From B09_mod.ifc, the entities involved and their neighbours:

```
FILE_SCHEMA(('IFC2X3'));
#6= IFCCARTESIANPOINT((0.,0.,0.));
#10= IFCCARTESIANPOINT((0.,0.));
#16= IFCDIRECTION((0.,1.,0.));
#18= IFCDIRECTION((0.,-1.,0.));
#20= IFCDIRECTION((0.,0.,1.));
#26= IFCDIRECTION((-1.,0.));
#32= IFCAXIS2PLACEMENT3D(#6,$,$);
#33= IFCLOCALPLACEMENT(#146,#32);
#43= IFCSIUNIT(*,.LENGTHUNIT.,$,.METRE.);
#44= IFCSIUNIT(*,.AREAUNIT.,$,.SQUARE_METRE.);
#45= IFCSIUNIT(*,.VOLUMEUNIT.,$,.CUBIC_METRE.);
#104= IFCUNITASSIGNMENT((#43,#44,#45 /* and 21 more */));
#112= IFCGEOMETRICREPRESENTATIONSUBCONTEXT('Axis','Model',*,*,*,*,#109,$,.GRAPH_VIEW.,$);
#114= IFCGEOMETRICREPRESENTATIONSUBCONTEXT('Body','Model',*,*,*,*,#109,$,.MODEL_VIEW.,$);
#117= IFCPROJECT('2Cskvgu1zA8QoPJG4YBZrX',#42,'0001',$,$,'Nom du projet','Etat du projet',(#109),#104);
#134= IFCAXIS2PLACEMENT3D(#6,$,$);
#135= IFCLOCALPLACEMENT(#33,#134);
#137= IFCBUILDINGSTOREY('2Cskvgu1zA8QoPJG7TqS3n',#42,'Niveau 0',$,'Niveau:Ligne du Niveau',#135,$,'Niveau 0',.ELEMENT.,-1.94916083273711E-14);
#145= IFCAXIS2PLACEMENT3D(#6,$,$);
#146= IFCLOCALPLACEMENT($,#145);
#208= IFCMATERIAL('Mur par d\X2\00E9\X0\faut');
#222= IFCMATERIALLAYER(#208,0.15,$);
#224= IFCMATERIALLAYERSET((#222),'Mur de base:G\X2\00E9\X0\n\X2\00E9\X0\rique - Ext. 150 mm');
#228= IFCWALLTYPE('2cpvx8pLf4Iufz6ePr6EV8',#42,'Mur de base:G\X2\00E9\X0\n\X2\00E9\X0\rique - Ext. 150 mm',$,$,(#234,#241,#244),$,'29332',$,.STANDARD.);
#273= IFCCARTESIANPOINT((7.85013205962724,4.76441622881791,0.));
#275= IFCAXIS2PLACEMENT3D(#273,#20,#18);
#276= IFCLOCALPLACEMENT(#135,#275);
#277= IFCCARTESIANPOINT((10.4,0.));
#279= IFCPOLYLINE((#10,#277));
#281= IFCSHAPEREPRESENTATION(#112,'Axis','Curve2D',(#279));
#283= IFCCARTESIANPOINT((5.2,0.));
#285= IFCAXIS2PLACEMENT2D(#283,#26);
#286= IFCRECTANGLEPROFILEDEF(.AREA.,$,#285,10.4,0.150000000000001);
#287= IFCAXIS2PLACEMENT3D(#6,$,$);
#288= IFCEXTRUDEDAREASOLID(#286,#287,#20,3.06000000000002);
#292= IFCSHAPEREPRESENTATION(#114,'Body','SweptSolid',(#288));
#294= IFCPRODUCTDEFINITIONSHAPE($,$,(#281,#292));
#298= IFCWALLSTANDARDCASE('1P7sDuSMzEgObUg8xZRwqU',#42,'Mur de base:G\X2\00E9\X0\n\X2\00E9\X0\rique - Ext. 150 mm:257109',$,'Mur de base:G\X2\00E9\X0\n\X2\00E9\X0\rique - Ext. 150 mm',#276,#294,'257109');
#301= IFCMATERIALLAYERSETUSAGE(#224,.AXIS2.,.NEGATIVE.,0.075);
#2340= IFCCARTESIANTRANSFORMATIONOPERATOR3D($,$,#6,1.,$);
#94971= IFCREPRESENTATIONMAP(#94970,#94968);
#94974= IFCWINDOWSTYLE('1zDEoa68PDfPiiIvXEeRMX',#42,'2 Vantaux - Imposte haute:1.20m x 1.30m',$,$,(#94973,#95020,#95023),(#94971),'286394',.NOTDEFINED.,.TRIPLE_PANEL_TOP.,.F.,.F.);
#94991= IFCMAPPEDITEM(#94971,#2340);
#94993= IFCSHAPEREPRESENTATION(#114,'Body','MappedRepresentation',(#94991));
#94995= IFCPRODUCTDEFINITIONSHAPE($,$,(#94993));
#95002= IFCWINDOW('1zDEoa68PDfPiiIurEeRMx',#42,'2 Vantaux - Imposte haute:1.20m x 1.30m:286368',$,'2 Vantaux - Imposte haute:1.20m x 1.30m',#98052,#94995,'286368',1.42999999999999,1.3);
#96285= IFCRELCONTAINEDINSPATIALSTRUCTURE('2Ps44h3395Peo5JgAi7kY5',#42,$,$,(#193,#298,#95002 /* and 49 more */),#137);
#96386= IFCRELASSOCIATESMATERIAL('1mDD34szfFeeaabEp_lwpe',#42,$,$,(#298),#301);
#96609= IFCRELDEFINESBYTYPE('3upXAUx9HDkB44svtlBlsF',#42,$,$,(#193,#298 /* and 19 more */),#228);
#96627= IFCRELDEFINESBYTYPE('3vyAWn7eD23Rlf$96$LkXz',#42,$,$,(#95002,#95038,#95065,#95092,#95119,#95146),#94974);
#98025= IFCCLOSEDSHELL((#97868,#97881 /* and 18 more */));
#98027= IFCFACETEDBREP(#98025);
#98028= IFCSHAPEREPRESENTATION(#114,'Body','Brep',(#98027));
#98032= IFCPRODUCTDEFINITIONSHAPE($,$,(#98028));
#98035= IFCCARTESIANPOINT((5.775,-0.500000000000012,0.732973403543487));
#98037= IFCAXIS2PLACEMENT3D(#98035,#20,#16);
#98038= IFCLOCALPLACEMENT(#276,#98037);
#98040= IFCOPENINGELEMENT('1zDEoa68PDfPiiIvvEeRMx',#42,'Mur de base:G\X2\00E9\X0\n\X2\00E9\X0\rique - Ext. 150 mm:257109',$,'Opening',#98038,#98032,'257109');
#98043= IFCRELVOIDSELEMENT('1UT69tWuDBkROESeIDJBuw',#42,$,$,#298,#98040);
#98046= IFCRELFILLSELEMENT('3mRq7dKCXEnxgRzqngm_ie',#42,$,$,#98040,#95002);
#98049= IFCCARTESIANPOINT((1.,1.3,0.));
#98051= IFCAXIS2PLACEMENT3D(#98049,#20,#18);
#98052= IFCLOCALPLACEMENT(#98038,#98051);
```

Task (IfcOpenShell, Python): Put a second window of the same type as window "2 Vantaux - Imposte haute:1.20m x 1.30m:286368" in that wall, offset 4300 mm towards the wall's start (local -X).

```python
import ifcopenshell
import ifcopenshell.api.feature
import ifcopenshell.api.geometry
import ifcopenshell.api.root
import ifcopenshell.geom
import ifcopenshell.util.element
import ifcopenshell.util.placement
import ifcopenshell.util.shape
import ifcopenshell.util.unit

model = ifcopenshell.open("B09_mod.ifc")
unit_scale = ifcopenshell.util.unit.calculate_unit_scale(model)
settings = ifcopenshell.geom.settings()


def volume(element):
    """Net volume in cubic metres, openings subtracted."""
    shape = ifcopenshell.geom.create_shape(settings, element)
    return ifcopenshell.util.shape.get_volume(shape.geometry)


def reuse_history(source, copy):
    """copy_class also copies each property set's owner history, people and application; keep the originals."""
    for rel in copy.IsDefinedBy:
        if rel.is_a("IfcRelDefinesByProperties") and (history := rel.RelatingPropertyDefinition.OwnerHistory):
            rel.RelatingPropertyDefinition.OwnerHistory = source.OwnerHistory
            ifcopenshell.util.element.remove_deep2(model, history)


window = model.by_guid("1zDEoa68PDfPiiIurEeRMx")
opening = window.FillsVoids[0].RelatingOpeningElement
wall = opening.VoidsElements[0].RelatingBuildingElement
before = volume(wall)
shift = ifcopenshell.util.placement.get_local_placement(wall.ObjectPlacement)[:3, 0] * -4.3 / unit_scale

# copy_class copies the void relationship, type, container and properties, but no geometry.
new_opening = ifcopenshell.api.root.copy_class(model, product=opening)
new_opening.Representation = ifcopenshell.util.element.copy_deep(
    model, opening.Representation, exclude=["IfcGeometricRepresentationContext", "IfcRepresentationMap"]
)
new_opening.Name = "Mur de base:Générique - Ext. 150 mm"
new_opening.Tag = None
new_window = ifcopenshell.api.root.copy_class(model, product=window)
new_window.Representation = ifcopenshell.util.element.copy_deep(
    model, window.Representation, exclude=["IfcGeometricRepresentationContext", "IfcRepresentationMap"]
)
new_window.Name = "2 Vantaux - Imposte haute:1.20m x 1.30m"
new_window.Tag = None
reuse_history(window, new_window)
fills = ifcopenshell.api.feature.add_filling(model, opening=new_opening, element=new_window)
fills.OwnerHistory = new_window.OwnerHistory  # required in IFC2X3

for old, new in ((opening, new_opening), (window, new_window)):
    matrix = ifcopenshell.util.placement.get_local_placement(old.ObjectPlacement)
    matrix[:3, 3] += shift
    ifcopenshell.api.geometry.edit_object_placement(model, product=new, matrix=matrix, is_si=False)

after = volume(wall)

print(f"wall volume {before:.3f} -> {after:.3f} m3")

model.write("B09_mod_rev.ifc")
```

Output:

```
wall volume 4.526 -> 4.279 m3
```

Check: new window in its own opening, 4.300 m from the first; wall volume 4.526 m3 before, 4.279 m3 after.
